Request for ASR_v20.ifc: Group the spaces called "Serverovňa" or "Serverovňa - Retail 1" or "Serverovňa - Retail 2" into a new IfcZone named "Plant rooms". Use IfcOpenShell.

First a look at what the model holds.

```python
import ifcopenshell

model = ifcopenshell.open("ASR_v20.ifc")
print(model.schema)
seen = {}
for space in model.by_type("IfcSpace"):
    seen[space.LongName] = seen.get(space.LongName, 0) + 1
for name, count in sorted(seen.items(), key=str):
    print(count, "x", name)
print("zones:", [z.Name for z in model.by_type("IfcZone")][:20])
```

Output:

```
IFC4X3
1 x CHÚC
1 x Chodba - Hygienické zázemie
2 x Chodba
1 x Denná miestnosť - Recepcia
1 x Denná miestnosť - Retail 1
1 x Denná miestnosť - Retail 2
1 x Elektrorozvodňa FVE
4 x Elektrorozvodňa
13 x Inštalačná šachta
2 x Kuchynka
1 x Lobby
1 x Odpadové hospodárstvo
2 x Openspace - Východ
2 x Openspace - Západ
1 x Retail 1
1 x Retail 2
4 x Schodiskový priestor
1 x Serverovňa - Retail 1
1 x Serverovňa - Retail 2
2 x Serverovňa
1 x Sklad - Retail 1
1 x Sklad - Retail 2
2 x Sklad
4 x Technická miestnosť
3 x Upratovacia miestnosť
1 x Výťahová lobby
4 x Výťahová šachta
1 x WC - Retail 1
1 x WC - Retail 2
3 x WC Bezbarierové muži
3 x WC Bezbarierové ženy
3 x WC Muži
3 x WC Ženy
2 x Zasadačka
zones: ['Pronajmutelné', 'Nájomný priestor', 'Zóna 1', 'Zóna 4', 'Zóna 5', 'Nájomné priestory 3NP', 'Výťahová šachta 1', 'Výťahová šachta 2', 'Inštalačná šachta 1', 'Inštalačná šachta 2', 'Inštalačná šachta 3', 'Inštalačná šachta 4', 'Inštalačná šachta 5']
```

```python
import ifcopenshell
import ifcopenshell.api.group
import ifcopenshell.api.root

model = ifcopenshell.open("ASR_v20.ifc")

names = {"Serverovňa", "Serverovňa - Retail 1", "Serverovňa - Retail 2"}
spaces = [s for s in model.by_type("IfcSpace") if s.LongName in names]

zone = ifcopenshell.api.root.create_entity(model, ifc_class="IfcZone", name="Plant rooms")
ifcopenshell.api.group.assign_group(model, products=spaces, group=zone)
print(len(spaces), "spaces in", zone.Name)

model.write("ASR_v20_rev.ifc")
```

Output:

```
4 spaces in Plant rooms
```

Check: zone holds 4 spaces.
